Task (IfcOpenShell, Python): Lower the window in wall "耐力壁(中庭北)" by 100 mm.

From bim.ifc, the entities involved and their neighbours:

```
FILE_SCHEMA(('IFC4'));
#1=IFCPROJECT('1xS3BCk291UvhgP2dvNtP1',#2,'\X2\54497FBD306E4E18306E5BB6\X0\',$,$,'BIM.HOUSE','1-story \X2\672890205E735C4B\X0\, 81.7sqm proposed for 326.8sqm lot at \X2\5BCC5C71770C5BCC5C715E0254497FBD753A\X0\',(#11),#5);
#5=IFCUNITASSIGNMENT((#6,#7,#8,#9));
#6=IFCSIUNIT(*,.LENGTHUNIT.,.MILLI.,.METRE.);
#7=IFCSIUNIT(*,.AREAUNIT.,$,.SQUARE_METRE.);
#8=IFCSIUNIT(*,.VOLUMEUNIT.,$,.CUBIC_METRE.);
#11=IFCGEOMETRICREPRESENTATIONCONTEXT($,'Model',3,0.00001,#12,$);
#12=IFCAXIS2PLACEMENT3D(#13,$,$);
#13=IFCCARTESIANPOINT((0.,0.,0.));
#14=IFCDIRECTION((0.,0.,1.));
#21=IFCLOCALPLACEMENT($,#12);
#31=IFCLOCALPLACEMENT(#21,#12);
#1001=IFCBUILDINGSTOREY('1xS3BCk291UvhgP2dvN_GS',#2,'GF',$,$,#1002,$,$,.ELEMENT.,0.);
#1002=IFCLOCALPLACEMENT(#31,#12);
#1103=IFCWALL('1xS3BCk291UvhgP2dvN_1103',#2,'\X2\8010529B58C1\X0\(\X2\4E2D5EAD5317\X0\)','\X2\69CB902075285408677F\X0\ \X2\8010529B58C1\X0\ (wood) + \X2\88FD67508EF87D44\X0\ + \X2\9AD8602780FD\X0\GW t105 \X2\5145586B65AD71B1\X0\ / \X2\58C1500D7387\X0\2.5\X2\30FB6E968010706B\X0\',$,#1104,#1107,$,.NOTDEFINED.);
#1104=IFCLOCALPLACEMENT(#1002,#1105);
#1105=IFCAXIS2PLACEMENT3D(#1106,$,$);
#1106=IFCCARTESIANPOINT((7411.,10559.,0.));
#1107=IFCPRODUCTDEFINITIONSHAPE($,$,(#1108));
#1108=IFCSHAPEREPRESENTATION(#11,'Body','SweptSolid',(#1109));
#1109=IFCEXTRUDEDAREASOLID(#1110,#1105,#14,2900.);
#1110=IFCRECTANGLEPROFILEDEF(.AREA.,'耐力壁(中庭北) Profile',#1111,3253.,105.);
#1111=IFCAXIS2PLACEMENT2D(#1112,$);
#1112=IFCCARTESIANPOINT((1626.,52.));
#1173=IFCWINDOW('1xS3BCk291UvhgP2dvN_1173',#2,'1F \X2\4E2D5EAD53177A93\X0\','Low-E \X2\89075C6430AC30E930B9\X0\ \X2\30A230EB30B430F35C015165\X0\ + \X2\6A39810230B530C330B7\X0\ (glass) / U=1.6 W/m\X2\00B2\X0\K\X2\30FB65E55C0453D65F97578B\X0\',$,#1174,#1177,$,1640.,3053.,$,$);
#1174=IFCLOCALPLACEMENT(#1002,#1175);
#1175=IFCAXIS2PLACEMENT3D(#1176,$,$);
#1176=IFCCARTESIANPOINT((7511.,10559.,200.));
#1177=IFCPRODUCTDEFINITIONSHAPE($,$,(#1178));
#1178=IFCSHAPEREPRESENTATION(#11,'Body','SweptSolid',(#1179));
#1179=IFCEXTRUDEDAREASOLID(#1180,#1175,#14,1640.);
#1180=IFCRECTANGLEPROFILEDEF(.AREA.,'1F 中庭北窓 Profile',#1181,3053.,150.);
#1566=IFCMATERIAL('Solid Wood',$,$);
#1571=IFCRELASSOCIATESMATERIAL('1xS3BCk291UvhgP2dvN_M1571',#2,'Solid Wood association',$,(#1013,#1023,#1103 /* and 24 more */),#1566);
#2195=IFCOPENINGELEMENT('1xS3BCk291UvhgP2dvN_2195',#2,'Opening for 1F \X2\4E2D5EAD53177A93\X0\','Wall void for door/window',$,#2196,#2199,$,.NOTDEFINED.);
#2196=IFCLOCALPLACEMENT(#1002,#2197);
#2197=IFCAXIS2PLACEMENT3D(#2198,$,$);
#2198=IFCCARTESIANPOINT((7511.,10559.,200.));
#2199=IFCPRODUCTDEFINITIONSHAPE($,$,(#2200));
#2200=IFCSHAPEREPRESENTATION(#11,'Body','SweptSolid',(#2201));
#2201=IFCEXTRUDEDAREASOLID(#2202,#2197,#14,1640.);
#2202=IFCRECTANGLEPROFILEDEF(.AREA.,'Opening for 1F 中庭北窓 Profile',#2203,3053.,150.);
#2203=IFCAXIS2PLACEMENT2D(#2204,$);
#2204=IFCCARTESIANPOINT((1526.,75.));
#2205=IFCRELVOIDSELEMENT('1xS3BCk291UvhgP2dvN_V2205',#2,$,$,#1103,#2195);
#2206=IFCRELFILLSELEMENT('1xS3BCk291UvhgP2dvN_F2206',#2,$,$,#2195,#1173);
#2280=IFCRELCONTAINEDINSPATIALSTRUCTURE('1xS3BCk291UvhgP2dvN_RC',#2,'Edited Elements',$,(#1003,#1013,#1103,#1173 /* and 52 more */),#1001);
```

```python
import numpy as np
import ifcopenshell
import ifcopenshell.api.geometry
import ifcopenshell.util.placement
import ifcopenshell.util.unit

model = ifcopenshell.open("bim.ifc")
unit_scale = ifcopenshell.util.unit.calculate_unit_scale(model)

window = model.by_id(1173)
opening = window.FillsVoids[0].RelatingOpeningElement
dz = -0.1 / unit_scale

shift = np.array([0.0, 0.0, dz])
# The window is not placed relative to its opening, so move both.
for product in (opening, window):
    matrix = ifcopenshell.util.placement.get_local_placement(product.ObjectPlacement)
    matrix[:3, 3] += shift
    ifcopenshell.api.geometry.edit_object_placement(model, product=product, matrix=matrix, is_si=False)

print(f"moved by {dz * unit_scale:+.3f} m")

model.write("bim_v2.ifc")
```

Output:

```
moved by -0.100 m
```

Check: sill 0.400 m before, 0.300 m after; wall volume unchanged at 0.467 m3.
